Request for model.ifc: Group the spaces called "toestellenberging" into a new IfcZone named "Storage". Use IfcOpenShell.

First a look at what the model holds.

```python
import ifcopenshell

model = ifcopenshell.open("model.ifc")
print(model.schema)
seen = {}
for space in model.by_type("IfcSpace"):
    seen[space.LongName] = seen.get(space.LongName, 0) + 1
for name, count in sorted(seen.items(), key=str):
    print(count, "x", name)
print("zones:", [z.Name for z in model.by_type("IfcZone")][:20])
```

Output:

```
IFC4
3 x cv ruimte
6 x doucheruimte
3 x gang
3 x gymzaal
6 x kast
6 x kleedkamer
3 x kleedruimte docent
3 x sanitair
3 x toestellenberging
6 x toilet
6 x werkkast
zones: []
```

```python
import ifcopenshell
import ifcopenshell.api.group
import ifcopenshell.api.root

model = ifcopenshell.open("model.ifc")

names = {"toestellenberging"}
spaces = [s for s in model.by_type("IfcSpace") if s.LongName in names]

zone = ifcopenshell.api.root.create_entity(model, ifc_class="IfcZone", name="Storage")
ifcopenshell.api.group.assign_group(model, products=spaces, group=zone)
print(len(spaces), "spaces in", zone.Name)

model.write("model-out.ifc")
```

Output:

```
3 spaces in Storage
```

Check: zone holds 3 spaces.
